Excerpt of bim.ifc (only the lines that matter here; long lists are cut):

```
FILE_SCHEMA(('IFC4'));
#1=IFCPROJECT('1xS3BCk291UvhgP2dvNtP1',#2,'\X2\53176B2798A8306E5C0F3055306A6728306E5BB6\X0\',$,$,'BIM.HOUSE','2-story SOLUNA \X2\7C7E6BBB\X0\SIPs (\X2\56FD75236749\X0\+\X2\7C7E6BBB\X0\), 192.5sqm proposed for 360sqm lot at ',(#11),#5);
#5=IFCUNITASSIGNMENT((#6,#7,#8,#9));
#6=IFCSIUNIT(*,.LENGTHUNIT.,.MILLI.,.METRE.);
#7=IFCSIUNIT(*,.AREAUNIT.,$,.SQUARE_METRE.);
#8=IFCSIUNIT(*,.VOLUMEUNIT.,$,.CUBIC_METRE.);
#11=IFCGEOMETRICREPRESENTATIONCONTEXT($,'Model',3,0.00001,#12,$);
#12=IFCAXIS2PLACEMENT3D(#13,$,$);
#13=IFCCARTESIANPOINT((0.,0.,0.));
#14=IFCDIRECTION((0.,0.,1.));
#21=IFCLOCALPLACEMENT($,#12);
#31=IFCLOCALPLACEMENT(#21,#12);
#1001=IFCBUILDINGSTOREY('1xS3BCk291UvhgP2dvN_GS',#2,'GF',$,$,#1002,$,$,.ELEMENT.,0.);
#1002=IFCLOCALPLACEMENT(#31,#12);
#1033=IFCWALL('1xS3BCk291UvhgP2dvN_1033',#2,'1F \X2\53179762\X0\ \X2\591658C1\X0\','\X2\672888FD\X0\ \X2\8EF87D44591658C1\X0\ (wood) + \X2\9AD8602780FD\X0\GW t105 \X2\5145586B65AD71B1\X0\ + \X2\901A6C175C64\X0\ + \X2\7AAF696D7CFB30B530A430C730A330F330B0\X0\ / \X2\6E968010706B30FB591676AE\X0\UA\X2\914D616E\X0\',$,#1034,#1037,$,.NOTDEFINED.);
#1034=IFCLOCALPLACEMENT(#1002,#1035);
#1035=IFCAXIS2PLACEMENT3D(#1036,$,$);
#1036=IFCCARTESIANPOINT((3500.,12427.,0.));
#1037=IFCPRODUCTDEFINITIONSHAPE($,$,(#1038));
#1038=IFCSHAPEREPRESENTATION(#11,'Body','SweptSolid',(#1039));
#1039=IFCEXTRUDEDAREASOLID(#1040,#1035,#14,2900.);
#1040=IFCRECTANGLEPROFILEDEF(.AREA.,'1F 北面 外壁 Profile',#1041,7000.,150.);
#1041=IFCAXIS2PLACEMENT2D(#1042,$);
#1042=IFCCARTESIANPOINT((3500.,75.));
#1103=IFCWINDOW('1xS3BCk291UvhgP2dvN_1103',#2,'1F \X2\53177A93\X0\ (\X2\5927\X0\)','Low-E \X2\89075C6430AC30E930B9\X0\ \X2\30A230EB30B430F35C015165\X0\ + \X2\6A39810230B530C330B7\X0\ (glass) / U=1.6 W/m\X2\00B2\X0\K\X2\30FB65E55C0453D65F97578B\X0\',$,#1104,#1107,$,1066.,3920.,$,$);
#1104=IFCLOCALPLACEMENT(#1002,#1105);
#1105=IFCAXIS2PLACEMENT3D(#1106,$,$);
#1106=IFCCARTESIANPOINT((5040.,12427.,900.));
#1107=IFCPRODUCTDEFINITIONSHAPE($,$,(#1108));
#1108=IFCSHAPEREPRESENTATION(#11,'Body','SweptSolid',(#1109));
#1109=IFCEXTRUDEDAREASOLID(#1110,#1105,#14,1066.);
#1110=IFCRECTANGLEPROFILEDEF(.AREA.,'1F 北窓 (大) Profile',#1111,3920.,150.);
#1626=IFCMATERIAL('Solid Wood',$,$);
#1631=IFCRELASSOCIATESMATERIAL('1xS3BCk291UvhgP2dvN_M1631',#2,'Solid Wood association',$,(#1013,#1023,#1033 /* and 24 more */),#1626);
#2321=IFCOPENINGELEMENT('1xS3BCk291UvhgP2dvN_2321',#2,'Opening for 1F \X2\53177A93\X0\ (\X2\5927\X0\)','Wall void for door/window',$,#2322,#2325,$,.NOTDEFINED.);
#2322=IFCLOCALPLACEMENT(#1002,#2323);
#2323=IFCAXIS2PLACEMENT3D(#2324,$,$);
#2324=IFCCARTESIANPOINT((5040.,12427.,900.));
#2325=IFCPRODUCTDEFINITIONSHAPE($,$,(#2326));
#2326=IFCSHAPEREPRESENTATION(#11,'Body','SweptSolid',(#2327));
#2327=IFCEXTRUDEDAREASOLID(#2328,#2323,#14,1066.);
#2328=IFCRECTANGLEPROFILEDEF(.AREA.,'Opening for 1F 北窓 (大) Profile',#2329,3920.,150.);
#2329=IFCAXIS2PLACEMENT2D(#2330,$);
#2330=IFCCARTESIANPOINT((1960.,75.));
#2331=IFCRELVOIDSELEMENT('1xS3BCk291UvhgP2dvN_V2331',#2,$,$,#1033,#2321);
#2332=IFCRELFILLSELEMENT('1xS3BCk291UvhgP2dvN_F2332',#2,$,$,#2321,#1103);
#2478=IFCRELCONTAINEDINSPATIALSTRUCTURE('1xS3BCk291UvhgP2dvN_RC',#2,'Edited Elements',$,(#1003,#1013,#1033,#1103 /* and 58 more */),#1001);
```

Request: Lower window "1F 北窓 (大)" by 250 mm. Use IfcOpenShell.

```python
import numpy as np
import ifcopenshell
import ifcopenshell.api.geometry
import ifcopenshell.util.placement
import ifcopenshell.util.unit

model = ifcopenshell.open("bim.ifc")
unit_scale = ifcopenshell.util.unit.calculate_unit_scale(model)

window = model.by_guid("1xS3BCk291UvhgP2dvN_1103")
opening = window.FillsVoids[0].RelatingOpeningElement
dz = -0.25 / unit_scale

shift = np.array([0.0, 0.0, dz])
# The window is not placed relative to its opening, so move both.
for product in (opening, window):
    matrix = ifcopenshell.util.placement.get_local_placement(product.ObjectPlacement)
    matrix[:3, 3] += shift
    ifcopenshell.api.geometry.edit_object_placement(model, product=product, matrix=matrix, is_si=False)

print(f"moved by {dz * unit_scale:+.3f} m")

model.write("bim_updated.ifc")
```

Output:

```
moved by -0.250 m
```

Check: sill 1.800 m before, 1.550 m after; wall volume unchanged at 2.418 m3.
